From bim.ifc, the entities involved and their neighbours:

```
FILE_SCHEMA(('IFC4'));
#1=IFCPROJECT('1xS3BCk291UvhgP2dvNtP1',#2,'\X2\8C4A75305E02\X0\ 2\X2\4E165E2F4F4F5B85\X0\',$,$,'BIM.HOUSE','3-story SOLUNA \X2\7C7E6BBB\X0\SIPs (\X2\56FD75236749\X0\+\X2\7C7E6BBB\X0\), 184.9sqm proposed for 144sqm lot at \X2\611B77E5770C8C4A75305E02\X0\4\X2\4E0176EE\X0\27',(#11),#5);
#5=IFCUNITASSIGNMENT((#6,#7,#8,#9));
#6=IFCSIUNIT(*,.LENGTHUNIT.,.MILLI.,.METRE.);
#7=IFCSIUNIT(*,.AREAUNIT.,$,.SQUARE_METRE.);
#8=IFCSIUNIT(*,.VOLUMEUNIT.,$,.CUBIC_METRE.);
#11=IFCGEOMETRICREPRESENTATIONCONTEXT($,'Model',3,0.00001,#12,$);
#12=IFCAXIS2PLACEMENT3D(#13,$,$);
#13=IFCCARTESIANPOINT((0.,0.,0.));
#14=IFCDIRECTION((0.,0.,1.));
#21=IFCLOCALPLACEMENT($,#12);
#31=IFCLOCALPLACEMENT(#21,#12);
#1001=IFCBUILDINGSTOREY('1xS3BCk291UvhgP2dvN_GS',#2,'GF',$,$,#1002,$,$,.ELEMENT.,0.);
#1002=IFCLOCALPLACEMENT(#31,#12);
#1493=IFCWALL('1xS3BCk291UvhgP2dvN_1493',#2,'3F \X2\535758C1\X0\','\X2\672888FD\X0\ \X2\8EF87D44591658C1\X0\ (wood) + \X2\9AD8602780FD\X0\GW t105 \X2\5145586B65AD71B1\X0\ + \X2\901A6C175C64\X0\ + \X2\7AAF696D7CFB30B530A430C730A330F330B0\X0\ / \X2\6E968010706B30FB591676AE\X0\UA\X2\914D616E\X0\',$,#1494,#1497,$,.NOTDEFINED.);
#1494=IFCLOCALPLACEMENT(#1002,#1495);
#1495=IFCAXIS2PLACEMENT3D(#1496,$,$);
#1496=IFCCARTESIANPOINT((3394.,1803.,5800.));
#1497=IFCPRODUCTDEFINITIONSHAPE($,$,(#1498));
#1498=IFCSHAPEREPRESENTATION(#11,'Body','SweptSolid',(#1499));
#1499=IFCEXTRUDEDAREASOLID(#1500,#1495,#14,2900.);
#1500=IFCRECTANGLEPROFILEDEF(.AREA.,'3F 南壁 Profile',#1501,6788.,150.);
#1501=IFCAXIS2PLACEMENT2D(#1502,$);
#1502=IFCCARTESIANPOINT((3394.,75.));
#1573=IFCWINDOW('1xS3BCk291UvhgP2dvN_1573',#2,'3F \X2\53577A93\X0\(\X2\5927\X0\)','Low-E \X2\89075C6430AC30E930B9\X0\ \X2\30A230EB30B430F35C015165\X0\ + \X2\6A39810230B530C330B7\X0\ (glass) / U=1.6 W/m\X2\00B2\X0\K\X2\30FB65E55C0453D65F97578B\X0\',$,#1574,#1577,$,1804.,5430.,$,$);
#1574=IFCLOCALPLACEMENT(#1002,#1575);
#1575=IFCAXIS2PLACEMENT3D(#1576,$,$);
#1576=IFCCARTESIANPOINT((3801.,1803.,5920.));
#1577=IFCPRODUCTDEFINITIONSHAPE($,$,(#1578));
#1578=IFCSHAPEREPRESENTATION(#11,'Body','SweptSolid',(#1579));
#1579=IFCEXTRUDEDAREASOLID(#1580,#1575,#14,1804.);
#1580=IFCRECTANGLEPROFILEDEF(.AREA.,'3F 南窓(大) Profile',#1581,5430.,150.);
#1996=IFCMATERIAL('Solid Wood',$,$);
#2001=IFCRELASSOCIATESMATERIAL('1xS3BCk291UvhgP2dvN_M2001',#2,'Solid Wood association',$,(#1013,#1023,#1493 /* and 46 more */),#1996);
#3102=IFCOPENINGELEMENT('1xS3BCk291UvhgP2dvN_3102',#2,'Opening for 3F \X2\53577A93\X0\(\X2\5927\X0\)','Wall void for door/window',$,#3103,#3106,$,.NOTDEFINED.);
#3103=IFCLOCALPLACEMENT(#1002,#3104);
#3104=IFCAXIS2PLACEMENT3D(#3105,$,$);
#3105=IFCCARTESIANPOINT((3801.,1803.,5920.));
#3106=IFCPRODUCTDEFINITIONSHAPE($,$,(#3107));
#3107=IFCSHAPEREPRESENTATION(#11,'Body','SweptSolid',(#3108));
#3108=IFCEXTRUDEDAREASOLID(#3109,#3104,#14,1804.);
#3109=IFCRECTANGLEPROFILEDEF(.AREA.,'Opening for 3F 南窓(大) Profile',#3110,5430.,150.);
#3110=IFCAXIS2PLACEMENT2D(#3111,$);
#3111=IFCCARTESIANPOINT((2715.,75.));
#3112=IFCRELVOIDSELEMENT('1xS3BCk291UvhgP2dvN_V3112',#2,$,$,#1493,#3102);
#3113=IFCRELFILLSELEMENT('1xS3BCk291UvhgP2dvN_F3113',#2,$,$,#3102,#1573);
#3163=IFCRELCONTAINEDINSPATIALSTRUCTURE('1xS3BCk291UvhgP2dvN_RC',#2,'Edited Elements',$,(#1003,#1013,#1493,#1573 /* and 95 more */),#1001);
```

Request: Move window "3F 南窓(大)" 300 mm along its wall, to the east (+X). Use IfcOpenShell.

```python
import ifcopenshell
import ifcopenshell.api.geometry
import ifcopenshell.util.placement

model = ifcopenshell.open("bim.ifc")

window = model.by_guid("1xS3BCk291UvhgP2dvN_1573")
opening = window.FillsVoids[0].RelatingOpeningElement
wall = opening.VoidsElements[0].RelatingBuildingElement

wall_matrix = ifcopenshell.util.placement.get_local_placement(wall.ObjectPlacement)
shift = wall_matrix[:3, 0] * 300.0
before = ifcopenshell.util.placement.get_local_placement(window.ObjectPlacement)[:3, 3].copy()

# The window is not placed relative to its opening, so move both.
for product in (opening, window):
    matrix = ifcopenshell.util.placement.get_local_placement(product.ObjectPlacement)
    matrix[:3, 3] += shift
    ifcopenshell.api.geometry.edit_object_placement(model, product=product, matrix=matrix, is_si=False)

after = ifcopenshell.util.placement.get_local_placement(window.ObjectPlacement)[:3, 3]
print("window moved by", (after - before).round(3) + 0.0)

model.write("bim-out.ifc")
```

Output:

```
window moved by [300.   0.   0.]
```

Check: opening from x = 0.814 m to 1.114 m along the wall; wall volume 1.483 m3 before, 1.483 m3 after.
